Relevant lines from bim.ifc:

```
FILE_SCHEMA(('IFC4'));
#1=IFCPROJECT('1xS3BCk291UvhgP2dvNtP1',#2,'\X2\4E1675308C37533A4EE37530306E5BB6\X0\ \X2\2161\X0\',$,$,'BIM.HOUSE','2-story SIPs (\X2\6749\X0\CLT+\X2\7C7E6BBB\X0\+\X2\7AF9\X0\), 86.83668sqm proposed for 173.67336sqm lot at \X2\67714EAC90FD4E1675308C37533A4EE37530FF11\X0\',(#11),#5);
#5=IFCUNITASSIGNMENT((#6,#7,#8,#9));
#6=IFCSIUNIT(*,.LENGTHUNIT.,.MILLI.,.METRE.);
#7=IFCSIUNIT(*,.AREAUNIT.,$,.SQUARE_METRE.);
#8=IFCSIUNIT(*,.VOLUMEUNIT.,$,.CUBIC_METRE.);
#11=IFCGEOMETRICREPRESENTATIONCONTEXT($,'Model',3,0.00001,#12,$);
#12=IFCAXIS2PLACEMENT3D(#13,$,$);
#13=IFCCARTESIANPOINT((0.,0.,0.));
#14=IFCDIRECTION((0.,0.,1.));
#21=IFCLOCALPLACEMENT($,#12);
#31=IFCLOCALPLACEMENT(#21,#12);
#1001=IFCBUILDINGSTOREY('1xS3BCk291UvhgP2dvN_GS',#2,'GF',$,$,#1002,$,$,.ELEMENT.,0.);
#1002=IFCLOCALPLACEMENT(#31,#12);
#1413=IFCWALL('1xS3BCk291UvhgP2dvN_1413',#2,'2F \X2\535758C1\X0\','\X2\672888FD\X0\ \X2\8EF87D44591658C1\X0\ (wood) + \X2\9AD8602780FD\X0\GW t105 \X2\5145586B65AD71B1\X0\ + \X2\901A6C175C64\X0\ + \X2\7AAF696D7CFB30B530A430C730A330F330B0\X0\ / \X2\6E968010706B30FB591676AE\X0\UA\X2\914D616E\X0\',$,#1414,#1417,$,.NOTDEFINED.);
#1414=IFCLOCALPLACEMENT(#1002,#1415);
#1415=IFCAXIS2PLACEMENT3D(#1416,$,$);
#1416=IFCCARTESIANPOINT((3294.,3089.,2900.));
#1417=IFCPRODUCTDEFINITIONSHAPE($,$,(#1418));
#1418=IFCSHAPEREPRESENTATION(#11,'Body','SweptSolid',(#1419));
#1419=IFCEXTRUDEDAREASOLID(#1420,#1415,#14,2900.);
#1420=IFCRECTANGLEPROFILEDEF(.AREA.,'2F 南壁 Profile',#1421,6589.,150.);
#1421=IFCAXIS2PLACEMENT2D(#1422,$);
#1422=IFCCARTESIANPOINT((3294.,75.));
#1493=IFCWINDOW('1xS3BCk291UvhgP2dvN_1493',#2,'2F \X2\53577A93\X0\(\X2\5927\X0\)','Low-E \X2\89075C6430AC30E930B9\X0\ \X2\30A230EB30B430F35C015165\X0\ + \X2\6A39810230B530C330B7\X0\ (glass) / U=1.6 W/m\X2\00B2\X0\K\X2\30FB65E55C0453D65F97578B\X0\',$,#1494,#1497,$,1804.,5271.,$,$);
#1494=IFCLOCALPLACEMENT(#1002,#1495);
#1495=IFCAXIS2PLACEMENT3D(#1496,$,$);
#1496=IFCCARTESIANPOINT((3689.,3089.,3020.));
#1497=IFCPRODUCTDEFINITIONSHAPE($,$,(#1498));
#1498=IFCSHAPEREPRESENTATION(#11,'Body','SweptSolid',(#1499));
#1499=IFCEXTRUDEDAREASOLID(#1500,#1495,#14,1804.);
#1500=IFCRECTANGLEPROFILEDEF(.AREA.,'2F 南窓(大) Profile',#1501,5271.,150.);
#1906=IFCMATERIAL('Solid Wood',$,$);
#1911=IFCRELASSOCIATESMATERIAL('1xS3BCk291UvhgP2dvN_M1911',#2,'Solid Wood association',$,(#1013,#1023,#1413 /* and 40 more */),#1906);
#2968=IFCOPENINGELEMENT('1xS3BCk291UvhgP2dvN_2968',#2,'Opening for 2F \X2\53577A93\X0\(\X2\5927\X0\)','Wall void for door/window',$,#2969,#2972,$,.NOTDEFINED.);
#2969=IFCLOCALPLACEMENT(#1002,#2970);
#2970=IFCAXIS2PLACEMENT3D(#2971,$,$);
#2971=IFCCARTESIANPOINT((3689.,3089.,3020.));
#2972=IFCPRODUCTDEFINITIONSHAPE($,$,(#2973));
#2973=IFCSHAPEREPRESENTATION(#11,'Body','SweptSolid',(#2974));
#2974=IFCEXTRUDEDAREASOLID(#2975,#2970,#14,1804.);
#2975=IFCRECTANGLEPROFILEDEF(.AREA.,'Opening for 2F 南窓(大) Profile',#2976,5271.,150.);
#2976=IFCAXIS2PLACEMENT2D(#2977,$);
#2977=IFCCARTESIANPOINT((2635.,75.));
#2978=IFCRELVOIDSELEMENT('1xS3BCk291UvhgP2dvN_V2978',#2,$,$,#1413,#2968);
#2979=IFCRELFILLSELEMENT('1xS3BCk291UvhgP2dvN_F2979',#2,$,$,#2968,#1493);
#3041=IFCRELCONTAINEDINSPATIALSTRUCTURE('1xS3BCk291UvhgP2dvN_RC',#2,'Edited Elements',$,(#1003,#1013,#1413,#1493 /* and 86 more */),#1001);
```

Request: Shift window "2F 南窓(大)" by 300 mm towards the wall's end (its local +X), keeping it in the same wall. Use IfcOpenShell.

```python
import ifcopenshell
import ifcopenshell.api.geometry
import ifcopenshell.util.placement
import ifcopenshell.util.unit

model = ifcopenshell.open("bim.ifc")
unit_scale = ifcopenshell.util.unit.calculate_unit_scale(model)

window = model.by_id(1493)
opening = window.FillsVoids[0].RelatingOpeningElement
wall = opening.VoidsElements[0].RelatingBuildingElement

wall_matrix = ifcopenshell.util.placement.get_local_placement(wall.ObjectPlacement)
shift = wall_matrix[:3, 0] * 0.3 / unit_scale
before = ifcopenshell.util.placement.get_local_placement(window.ObjectPlacement)[:3, 3].copy()

# The window is not placed relative to its opening, so move both.
for product in (opening, window):
    matrix = ifcopenshell.util.placement.get_local_placement(product.ObjectPlacement)
    matrix[:3, 3] += shift
    ifcopenshell.api.geometry.edit_object_placement(model, product=product, matrix=matrix, is_si=False)

after = ifcopenshell.util.placement.get_local_placement(window.ObjectPlacement)[:3, 3]
print("window moved by", (after - before).round(3) + 0.0)

model.write("bim_v2.ifc")
```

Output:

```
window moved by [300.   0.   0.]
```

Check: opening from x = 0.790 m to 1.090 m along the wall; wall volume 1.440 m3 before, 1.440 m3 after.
